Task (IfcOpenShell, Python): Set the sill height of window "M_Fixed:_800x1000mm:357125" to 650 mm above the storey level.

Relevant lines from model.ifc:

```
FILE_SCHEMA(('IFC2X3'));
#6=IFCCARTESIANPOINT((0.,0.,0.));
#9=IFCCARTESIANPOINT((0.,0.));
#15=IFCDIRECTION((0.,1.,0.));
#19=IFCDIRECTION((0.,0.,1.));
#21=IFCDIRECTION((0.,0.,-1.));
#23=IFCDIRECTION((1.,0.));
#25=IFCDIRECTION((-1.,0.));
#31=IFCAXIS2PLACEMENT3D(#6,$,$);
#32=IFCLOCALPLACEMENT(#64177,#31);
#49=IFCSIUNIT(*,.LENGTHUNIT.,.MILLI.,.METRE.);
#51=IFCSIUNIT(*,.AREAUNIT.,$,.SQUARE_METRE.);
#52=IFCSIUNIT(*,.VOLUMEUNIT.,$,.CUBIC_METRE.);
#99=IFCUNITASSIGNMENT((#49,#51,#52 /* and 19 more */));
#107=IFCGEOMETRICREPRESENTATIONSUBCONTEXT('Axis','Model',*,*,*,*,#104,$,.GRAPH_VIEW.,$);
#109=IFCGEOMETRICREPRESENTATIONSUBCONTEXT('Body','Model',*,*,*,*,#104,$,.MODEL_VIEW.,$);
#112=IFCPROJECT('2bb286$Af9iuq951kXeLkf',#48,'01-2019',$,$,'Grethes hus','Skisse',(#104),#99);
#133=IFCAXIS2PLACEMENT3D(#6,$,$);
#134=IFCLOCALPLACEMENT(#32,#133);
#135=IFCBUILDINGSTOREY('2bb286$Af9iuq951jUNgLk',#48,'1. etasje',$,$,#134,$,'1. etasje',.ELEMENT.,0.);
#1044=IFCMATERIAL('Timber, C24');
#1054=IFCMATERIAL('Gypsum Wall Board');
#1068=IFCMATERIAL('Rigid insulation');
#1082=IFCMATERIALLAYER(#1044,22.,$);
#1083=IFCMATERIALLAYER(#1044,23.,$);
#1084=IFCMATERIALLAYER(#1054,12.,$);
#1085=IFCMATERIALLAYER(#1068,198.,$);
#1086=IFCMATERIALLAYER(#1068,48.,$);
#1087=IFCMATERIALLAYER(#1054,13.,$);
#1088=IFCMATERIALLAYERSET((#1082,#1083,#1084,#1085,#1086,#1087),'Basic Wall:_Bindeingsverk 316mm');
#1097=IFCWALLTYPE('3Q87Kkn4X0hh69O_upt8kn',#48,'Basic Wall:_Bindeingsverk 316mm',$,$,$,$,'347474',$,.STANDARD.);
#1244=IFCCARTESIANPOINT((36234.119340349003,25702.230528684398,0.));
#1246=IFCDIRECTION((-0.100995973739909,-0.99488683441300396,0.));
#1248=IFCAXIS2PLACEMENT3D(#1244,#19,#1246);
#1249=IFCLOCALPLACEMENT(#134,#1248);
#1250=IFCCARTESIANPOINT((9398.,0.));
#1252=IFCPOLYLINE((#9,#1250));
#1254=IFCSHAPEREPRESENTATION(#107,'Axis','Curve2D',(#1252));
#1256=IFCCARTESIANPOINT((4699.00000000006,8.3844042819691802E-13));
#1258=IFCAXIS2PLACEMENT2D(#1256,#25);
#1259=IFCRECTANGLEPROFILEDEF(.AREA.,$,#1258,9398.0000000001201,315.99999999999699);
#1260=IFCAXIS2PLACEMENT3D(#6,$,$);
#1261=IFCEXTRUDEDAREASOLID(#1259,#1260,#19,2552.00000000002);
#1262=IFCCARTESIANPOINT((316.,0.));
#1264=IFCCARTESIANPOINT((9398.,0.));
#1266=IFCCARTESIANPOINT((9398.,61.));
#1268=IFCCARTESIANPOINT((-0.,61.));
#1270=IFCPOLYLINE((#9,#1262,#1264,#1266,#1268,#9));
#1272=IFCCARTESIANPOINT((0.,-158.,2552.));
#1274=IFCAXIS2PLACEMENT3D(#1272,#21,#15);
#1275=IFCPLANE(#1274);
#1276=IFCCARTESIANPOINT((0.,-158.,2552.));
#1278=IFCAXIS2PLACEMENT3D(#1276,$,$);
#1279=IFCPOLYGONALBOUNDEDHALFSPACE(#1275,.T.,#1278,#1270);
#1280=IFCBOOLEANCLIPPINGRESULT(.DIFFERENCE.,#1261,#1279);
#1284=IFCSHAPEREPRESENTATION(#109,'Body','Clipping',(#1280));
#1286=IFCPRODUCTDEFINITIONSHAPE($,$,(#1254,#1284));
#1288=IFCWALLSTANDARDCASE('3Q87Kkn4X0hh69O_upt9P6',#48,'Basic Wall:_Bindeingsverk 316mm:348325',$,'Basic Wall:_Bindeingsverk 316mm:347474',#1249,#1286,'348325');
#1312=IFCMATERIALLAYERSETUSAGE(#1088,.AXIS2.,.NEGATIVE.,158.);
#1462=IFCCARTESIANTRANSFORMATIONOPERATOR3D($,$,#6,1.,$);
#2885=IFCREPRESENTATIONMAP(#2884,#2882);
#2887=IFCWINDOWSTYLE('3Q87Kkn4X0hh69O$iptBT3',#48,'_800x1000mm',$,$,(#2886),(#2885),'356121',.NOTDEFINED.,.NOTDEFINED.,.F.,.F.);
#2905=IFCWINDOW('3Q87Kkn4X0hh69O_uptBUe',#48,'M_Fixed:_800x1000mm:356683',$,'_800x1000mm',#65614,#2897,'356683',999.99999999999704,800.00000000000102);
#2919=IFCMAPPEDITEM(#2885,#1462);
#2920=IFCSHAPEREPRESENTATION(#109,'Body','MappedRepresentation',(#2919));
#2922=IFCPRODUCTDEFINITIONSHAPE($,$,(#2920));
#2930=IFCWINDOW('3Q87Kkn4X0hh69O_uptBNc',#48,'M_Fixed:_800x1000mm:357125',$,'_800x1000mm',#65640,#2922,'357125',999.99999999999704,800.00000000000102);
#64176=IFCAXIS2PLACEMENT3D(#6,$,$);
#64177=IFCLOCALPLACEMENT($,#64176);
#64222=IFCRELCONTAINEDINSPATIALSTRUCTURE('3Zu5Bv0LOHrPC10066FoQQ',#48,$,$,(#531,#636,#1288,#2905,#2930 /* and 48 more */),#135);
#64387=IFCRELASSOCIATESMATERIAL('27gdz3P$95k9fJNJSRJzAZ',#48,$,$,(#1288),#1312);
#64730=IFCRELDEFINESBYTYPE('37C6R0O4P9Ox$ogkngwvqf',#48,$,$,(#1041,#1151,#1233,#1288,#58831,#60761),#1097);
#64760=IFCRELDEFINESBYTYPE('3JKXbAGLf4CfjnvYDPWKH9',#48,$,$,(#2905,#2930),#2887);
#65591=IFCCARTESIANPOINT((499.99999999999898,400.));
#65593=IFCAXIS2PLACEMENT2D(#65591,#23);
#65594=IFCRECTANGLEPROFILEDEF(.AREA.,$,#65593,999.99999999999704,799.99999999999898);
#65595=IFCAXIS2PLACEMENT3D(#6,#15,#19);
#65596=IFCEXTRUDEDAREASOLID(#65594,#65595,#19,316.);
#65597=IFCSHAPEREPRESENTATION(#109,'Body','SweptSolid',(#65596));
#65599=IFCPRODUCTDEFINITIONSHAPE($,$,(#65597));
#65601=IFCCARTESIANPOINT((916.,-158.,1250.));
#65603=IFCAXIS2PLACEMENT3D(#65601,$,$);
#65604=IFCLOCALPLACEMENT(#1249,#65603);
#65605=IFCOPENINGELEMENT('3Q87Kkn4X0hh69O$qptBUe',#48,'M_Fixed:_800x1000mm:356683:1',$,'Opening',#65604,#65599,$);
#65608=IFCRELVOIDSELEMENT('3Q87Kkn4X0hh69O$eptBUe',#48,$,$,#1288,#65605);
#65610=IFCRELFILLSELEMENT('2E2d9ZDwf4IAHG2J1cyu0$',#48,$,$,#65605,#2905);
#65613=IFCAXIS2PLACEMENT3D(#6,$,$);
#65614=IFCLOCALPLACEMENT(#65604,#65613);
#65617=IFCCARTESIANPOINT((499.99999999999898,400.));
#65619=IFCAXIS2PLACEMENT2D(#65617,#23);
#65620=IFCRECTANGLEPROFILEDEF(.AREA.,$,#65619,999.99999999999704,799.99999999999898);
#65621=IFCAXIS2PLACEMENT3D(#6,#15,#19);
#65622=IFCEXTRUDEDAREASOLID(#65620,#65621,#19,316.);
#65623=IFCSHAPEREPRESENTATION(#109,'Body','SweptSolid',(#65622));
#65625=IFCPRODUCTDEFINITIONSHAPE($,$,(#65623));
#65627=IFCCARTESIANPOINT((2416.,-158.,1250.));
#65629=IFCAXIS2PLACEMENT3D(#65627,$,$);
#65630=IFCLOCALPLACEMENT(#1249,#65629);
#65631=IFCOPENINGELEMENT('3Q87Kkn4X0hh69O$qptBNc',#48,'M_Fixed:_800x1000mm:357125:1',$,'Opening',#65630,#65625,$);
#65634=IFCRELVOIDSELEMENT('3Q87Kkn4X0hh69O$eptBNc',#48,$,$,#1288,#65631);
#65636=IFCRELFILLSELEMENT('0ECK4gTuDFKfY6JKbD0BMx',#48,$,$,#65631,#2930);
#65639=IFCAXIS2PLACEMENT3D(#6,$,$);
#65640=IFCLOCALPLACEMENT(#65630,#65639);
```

```python
import numpy as np
import ifcopenshell
import ifcopenshell.api.geometry
import ifcopenshell.geom
import ifcopenshell.util.element
import ifcopenshell.util.placement
import ifcopenshell.util.shape
import ifcopenshell.util.unit

model = ifcopenshell.open("model.ifc")
unit_scale = ifcopenshell.util.unit.calculate_unit_scale(model)

window = model.by_guid("3Q87Kkn4X0hh69O_uptBNc")
opening = window.FillsVoids[0].RelatingOpeningElement
storey = ifcopenshell.util.element.get_container(window, ifc_class="IfcBuildingStorey")
level = ifcopenshell.util.placement.get_local_placement(storey.ObjectPlacement)[2, 3]

# The opening's origin need not be at the sill, so measure its lowest point.
shape = ifcopenshell.geom.create_shape(ifcopenshell.geom.settings(), opening)
bottom = ifcopenshell.util.shape.get_shape_bottom_elevation(shape, shape.geometry) / unit_scale
dz = level + 0.65 / unit_scale - bottom

shift = np.array([0.0, 0.0, dz])
# The window is placed relative to its opening, so it follows when the opening moves.
matrix = ifcopenshell.util.placement.get_local_placement(opening.ObjectPlacement)
matrix[:3, 3] += shift
ifcopenshell.api.geometry.edit_object_placement(
    model, product=opening, matrix=matrix, is_si=False, should_transform_children=True
)

print(f"moved by {dz * unit_scale:+.3f} m")

model.write("model-out.ifc")
```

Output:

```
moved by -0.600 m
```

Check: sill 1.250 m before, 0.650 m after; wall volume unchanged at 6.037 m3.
